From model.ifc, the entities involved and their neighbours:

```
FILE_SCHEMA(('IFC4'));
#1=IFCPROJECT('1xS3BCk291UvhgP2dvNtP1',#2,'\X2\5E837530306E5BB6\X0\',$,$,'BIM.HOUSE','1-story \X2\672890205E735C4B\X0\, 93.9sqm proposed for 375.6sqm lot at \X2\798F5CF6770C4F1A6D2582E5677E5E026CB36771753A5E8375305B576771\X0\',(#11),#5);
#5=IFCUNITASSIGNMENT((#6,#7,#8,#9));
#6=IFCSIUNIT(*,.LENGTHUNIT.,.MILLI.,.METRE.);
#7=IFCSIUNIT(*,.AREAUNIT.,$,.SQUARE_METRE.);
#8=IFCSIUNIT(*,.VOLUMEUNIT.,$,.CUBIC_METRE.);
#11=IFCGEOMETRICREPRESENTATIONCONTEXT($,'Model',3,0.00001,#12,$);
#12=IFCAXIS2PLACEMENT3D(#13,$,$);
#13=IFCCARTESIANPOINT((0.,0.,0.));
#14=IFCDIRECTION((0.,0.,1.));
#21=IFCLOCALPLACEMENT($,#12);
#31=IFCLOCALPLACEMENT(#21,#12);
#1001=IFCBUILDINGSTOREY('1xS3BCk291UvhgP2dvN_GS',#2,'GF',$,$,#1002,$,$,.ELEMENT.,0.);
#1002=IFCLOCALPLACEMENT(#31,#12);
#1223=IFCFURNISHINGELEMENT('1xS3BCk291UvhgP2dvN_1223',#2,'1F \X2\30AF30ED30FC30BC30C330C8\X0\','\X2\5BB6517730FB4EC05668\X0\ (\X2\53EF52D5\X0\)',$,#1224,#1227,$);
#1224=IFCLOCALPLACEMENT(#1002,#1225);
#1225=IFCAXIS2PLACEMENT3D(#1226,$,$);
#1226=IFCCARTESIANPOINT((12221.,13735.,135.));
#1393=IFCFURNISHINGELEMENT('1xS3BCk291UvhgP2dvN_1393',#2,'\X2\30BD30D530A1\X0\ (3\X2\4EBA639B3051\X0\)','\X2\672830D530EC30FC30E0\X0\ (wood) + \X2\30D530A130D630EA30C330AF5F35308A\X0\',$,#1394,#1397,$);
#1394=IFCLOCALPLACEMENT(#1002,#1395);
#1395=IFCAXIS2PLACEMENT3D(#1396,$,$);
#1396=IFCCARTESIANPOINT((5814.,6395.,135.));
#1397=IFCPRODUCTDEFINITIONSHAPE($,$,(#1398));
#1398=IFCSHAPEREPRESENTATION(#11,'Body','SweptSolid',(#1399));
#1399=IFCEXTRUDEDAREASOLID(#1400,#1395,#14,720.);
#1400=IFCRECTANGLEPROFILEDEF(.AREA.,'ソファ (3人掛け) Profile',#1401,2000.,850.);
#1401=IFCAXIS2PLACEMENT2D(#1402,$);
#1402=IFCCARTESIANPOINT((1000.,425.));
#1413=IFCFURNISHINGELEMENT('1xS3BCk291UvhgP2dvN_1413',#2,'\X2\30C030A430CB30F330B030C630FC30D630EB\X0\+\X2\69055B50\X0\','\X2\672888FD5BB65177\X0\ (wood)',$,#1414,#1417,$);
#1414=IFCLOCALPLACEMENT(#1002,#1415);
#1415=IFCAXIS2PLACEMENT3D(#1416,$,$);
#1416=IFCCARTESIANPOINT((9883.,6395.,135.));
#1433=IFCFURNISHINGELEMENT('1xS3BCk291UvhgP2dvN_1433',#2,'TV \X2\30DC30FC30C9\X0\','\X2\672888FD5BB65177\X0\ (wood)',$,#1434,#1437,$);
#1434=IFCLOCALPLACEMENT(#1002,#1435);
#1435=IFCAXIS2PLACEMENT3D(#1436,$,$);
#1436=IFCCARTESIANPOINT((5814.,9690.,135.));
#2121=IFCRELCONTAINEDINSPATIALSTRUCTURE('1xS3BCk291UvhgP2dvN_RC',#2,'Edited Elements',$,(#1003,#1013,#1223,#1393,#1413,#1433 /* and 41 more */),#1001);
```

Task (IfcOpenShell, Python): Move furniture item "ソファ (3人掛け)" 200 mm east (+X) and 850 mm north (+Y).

```python
import ifcopenshell
import ifcopenshell.api.geometry
import ifcopenshell.util.placement

model = ifcopenshell.open("model.ifc")

item = model.by_guid("1xS3BCk291UvhgP2dvN_1393")
matrix = ifcopenshell.util.placement.get_local_placement(item.ObjectPlacement)
matrix[0, 3] += 200.0
matrix[1, 3] += 850.0
ifcopenshell.api.geometry.edit_object_placement(model, product=item, matrix=matrix, is_si=False)

print(ifcopenshell.util.placement.get_local_placement(item.ObjectPlacement).round(3) + 0.0)

model.write("model_rev.ifc")
```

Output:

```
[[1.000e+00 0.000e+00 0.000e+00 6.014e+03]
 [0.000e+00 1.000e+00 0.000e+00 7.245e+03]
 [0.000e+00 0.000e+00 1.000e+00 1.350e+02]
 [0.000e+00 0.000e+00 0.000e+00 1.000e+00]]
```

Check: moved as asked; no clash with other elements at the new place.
